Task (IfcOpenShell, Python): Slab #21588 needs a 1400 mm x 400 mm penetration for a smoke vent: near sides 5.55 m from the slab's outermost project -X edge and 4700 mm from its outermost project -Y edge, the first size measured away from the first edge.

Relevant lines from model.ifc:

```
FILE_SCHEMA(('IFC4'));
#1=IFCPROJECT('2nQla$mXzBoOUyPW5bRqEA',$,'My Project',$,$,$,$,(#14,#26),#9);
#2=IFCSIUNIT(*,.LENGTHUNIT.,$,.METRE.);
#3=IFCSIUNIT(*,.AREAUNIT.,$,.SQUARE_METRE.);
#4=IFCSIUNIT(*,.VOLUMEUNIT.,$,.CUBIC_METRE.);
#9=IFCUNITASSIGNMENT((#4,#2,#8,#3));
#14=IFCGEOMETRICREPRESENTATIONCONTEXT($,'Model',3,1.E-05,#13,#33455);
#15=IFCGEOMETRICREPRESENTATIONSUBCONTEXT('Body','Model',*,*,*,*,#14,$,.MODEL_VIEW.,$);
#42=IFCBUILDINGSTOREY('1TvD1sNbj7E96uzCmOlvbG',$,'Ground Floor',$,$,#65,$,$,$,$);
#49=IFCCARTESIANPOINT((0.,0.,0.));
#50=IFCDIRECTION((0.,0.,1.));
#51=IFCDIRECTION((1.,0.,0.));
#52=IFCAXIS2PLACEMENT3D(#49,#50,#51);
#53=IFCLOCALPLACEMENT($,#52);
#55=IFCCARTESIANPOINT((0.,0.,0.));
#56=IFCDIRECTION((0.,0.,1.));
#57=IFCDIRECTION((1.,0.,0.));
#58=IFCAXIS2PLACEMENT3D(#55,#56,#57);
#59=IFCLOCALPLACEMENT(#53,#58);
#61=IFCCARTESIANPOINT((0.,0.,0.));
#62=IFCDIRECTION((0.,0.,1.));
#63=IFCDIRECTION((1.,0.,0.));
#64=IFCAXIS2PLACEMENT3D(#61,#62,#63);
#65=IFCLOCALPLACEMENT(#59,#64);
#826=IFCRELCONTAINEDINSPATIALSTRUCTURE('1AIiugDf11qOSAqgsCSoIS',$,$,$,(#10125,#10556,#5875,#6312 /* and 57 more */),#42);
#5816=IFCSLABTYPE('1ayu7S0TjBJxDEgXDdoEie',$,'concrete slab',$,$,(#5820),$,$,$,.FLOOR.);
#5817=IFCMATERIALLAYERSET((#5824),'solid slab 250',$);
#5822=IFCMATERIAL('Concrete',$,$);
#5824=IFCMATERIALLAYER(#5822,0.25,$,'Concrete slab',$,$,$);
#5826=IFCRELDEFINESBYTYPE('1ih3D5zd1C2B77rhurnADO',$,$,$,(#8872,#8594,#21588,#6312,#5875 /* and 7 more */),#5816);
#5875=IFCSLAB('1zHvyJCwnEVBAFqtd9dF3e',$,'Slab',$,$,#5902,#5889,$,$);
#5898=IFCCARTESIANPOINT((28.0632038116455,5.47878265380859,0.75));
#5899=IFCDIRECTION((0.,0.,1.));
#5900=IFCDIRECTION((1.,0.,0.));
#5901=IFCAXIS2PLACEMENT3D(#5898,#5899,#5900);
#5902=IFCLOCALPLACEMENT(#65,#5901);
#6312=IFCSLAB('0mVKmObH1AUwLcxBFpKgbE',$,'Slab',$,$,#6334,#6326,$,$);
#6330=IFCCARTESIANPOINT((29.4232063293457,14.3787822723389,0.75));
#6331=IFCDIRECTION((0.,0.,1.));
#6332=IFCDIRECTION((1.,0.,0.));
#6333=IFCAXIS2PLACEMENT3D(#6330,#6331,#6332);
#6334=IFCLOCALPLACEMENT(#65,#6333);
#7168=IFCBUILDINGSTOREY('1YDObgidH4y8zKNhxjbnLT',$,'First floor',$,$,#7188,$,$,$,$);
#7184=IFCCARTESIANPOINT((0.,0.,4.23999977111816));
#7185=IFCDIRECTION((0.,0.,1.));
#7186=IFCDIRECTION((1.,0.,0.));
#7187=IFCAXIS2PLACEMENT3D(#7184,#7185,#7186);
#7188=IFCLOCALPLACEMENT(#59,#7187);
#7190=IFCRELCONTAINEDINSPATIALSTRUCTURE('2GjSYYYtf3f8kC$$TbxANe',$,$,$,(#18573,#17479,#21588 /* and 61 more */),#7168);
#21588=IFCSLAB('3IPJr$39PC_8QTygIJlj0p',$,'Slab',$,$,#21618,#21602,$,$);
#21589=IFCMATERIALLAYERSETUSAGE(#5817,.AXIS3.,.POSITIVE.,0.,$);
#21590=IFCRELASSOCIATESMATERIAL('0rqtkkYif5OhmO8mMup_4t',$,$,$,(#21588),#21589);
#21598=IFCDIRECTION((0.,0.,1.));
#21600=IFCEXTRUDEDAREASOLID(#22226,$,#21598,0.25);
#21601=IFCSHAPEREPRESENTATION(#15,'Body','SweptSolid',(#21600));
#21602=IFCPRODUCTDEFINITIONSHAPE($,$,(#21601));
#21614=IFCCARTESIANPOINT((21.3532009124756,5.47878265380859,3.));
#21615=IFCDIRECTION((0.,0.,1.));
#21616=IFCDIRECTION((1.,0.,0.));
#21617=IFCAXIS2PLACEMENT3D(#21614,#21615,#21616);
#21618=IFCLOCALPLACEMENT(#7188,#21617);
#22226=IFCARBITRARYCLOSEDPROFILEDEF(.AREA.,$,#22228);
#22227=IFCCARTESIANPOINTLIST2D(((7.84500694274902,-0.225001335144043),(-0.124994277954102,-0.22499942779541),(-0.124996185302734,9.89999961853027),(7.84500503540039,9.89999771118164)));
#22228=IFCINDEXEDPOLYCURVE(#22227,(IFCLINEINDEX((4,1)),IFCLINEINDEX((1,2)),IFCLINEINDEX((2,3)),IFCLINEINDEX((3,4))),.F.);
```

```python
import numpy as np
import ifcopenshell
import ifcopenshell.api.feature
import ifcopenshell.api.geometry
import ifcopenshell.api.root
import ifcopenshell.geom
import ifcopenshell.util.placement
import ifcopenshell.util.representation
import ifcopenshell.util.shape
import ifcopenshell.util.unit

model = ifcopenshell.open("model.ifc")
unit_scale = ifcopenshell.util.unit.calculate_unit_scale(model)
settings = ifcopenshell.geom.settings()


def volume(element):
    """Net volume in cubic metres, openings subtracted."""
    shape = ifcopenshell.geom.create_shape(settings, element)
    return ifcopenshell.util.shape.get_volume(shape.geometry)


slab = model.by_guid("3IPJr$39PC_8QTygIJlj0p")
before = volume(slab)

# Extent in the slab's own axes, in metres. The edges named are its -X and -Y sides.
slab_shape = ifcopenshell.geom.create_shape(settings, slab)
vertices = ifcopenshell.util.shape.get_vertices(slab_shape.geometry)
x_min, y_min, bottom = vertices.min(axis=0)
top = vertices[:, 2].max()

opening = ifcopenshell.api.root.create_entity(model, ifc_class="IfcOpeningElement", name="Smoke vent opening", predefined_type="OPENING")
context = ifcopenshell.util.representation.get_context(model, "Model", "Body", "MODEL_VIEW")
width, depth = 1.4, 0.4
outline = [(0.0, 0.0), (width, 0.0), (width, depth), (0.0, depth), (0.0, 0.0)]
# Overshoot both faces by 50 mm so the cut is clean.
shape = ifcopenshell.api.geometry.add_slab_representation(
    model, context=context, depth=top - bottom + 0.1, polyline=outline
)
ifcopenshell.api.geometry.assign_representation(model, product=opening, representation=shape)

matrix = ifcopenshell.util.placement.get_local_placement(slab.ObjectPlacement)
matrix[:, 3] = matrix @ np.append(np.array([x_min + 5.55, y_min + 4.7, bottom - 0.05]) / unit_scale, 1.0)
ifcopenshell.api.geometry.edit_object_placement(model, product=opening, matrix=matrix, is_si=False)
ifcopenshell.api.feature.add_feature(model, feature=opening, element=slab)

after = volume(slab)

print(f"slab volume {before:.3f} -> {after:.3f} m3")

model.write("model_edited.ifc")
```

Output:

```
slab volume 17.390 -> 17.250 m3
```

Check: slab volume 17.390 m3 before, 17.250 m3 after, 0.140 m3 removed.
